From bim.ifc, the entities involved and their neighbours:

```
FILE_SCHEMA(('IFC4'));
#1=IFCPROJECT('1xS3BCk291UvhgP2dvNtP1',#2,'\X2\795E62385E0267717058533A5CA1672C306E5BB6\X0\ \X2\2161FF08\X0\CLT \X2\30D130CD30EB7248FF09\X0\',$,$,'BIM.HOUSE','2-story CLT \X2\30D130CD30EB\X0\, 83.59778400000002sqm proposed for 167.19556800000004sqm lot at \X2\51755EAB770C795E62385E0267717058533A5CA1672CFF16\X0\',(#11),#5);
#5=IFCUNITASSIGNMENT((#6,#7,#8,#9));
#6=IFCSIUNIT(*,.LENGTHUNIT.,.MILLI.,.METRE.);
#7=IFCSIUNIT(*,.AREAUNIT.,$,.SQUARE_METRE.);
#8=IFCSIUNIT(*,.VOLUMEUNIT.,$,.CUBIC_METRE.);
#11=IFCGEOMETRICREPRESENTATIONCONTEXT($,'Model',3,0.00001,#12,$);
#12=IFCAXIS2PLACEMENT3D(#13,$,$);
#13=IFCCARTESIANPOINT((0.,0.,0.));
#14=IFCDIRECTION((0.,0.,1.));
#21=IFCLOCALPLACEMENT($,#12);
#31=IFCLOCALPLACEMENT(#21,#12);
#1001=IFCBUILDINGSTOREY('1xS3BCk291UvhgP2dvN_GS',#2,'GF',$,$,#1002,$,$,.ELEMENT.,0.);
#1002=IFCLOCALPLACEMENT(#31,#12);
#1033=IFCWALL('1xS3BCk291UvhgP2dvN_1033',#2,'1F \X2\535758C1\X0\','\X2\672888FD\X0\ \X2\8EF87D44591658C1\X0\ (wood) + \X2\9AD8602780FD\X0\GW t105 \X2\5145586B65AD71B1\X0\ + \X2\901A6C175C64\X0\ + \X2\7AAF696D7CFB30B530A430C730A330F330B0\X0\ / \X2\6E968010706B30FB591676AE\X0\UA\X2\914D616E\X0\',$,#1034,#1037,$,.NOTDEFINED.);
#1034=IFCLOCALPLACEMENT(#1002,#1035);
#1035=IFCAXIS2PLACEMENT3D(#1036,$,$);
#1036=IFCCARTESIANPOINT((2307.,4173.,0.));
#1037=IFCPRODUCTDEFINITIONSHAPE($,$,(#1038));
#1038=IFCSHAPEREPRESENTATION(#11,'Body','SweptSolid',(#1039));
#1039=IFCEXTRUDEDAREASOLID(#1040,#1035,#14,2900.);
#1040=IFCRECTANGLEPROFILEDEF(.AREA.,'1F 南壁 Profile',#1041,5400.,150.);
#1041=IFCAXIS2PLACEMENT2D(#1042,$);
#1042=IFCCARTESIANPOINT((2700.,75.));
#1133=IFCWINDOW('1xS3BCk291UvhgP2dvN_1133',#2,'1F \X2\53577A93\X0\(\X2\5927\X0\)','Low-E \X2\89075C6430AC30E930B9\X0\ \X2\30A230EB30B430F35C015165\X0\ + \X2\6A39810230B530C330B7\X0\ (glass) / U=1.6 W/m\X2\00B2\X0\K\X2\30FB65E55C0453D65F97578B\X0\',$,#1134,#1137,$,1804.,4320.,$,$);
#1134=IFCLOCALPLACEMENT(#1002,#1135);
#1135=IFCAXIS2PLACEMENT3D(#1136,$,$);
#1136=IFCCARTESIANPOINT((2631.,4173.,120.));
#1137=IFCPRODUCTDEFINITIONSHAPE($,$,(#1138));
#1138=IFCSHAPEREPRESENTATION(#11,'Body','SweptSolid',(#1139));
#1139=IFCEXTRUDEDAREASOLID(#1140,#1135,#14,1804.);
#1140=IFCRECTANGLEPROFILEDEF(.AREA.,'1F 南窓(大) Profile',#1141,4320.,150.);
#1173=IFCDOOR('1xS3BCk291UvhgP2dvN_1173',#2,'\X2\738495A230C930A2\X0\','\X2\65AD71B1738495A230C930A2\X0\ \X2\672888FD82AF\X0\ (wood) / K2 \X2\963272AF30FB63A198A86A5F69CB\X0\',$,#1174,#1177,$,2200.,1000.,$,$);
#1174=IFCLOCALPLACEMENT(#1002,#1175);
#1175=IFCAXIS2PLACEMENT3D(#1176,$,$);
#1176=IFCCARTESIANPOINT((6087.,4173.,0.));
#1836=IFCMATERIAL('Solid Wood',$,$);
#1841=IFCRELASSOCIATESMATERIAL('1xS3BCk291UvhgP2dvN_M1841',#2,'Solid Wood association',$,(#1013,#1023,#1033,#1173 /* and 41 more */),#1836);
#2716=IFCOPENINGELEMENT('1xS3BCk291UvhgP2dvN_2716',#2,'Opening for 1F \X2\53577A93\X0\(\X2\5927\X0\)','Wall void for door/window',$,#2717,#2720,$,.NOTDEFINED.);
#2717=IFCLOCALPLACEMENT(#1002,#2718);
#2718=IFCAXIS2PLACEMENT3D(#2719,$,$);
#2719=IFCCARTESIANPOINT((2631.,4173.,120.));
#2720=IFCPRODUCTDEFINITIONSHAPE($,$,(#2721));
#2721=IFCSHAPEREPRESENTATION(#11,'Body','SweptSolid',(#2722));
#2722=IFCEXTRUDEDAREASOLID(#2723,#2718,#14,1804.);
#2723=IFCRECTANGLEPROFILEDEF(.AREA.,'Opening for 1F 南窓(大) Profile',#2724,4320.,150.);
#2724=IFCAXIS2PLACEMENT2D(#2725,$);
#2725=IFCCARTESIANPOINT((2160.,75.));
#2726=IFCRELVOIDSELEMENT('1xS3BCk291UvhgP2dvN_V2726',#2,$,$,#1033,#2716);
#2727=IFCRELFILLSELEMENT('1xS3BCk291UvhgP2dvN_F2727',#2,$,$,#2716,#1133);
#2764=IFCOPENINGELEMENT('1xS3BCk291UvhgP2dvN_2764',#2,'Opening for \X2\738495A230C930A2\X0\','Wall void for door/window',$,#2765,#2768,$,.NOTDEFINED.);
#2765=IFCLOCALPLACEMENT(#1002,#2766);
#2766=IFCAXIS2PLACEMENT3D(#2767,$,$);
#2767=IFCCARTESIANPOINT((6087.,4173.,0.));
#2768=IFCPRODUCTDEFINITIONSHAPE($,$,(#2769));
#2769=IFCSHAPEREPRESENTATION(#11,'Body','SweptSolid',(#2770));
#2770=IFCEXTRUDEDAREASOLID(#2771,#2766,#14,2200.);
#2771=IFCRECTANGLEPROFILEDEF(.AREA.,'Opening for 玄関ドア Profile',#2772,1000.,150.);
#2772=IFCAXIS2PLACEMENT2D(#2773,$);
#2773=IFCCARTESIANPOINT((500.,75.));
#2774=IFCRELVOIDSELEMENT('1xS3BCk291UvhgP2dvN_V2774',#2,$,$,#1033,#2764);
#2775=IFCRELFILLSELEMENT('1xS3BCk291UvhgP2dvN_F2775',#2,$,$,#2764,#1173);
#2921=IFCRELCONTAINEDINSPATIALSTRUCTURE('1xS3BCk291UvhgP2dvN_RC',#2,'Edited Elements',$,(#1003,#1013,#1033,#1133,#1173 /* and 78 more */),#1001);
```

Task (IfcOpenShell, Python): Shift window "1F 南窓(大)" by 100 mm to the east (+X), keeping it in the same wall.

```python
import ifcopenshell
import ifcopenshell.api.geometry
import ifcopenshell.util.placement
import ifcopenshell.util.unit

model = ifcopenshell.open("bim.ifc")
unit_scale = ifcopenshell.util.unit.calculate_unit_scale(model)

window = model.by_guid("1xS3BCk291UvhgP2dvN_1133")
opening = window.FillsVoids[0].RelatingOpeningElement
wall = opening.VoidsElements[0].RelatingBuildingElement

wall_matrix = ifcopenshell.util.placement.get_local_placement(wall.ObjectPlacement)
shift = wall_matrix[:3, 0] * 0.1 / unit_scale
before = ifcopenshell.util.placement.get_local_placement(window.ObjectPlacement)[:3, 3].copy()

# The window is not placed relative to its opening, so move both.
for product in (opening, window):
    matrix = ifcopenshell.util.placement.get_local_placement(product.ObjectPlacement)
    matrix[:3, 3] += shift
    ifcopenshell.api.geometry.edit_object_placement(model, product=product, matrix=matrix, is_si=False)

after = ifcopenshell.util.placement.get_local_placement(window.ObjectPlacement)[:3, 3]
print("window moved by", (after - before).round(3) + 0.0)

model.write("bim-out.ifc")
```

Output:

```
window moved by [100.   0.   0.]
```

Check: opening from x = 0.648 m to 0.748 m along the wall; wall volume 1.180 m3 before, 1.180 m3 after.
